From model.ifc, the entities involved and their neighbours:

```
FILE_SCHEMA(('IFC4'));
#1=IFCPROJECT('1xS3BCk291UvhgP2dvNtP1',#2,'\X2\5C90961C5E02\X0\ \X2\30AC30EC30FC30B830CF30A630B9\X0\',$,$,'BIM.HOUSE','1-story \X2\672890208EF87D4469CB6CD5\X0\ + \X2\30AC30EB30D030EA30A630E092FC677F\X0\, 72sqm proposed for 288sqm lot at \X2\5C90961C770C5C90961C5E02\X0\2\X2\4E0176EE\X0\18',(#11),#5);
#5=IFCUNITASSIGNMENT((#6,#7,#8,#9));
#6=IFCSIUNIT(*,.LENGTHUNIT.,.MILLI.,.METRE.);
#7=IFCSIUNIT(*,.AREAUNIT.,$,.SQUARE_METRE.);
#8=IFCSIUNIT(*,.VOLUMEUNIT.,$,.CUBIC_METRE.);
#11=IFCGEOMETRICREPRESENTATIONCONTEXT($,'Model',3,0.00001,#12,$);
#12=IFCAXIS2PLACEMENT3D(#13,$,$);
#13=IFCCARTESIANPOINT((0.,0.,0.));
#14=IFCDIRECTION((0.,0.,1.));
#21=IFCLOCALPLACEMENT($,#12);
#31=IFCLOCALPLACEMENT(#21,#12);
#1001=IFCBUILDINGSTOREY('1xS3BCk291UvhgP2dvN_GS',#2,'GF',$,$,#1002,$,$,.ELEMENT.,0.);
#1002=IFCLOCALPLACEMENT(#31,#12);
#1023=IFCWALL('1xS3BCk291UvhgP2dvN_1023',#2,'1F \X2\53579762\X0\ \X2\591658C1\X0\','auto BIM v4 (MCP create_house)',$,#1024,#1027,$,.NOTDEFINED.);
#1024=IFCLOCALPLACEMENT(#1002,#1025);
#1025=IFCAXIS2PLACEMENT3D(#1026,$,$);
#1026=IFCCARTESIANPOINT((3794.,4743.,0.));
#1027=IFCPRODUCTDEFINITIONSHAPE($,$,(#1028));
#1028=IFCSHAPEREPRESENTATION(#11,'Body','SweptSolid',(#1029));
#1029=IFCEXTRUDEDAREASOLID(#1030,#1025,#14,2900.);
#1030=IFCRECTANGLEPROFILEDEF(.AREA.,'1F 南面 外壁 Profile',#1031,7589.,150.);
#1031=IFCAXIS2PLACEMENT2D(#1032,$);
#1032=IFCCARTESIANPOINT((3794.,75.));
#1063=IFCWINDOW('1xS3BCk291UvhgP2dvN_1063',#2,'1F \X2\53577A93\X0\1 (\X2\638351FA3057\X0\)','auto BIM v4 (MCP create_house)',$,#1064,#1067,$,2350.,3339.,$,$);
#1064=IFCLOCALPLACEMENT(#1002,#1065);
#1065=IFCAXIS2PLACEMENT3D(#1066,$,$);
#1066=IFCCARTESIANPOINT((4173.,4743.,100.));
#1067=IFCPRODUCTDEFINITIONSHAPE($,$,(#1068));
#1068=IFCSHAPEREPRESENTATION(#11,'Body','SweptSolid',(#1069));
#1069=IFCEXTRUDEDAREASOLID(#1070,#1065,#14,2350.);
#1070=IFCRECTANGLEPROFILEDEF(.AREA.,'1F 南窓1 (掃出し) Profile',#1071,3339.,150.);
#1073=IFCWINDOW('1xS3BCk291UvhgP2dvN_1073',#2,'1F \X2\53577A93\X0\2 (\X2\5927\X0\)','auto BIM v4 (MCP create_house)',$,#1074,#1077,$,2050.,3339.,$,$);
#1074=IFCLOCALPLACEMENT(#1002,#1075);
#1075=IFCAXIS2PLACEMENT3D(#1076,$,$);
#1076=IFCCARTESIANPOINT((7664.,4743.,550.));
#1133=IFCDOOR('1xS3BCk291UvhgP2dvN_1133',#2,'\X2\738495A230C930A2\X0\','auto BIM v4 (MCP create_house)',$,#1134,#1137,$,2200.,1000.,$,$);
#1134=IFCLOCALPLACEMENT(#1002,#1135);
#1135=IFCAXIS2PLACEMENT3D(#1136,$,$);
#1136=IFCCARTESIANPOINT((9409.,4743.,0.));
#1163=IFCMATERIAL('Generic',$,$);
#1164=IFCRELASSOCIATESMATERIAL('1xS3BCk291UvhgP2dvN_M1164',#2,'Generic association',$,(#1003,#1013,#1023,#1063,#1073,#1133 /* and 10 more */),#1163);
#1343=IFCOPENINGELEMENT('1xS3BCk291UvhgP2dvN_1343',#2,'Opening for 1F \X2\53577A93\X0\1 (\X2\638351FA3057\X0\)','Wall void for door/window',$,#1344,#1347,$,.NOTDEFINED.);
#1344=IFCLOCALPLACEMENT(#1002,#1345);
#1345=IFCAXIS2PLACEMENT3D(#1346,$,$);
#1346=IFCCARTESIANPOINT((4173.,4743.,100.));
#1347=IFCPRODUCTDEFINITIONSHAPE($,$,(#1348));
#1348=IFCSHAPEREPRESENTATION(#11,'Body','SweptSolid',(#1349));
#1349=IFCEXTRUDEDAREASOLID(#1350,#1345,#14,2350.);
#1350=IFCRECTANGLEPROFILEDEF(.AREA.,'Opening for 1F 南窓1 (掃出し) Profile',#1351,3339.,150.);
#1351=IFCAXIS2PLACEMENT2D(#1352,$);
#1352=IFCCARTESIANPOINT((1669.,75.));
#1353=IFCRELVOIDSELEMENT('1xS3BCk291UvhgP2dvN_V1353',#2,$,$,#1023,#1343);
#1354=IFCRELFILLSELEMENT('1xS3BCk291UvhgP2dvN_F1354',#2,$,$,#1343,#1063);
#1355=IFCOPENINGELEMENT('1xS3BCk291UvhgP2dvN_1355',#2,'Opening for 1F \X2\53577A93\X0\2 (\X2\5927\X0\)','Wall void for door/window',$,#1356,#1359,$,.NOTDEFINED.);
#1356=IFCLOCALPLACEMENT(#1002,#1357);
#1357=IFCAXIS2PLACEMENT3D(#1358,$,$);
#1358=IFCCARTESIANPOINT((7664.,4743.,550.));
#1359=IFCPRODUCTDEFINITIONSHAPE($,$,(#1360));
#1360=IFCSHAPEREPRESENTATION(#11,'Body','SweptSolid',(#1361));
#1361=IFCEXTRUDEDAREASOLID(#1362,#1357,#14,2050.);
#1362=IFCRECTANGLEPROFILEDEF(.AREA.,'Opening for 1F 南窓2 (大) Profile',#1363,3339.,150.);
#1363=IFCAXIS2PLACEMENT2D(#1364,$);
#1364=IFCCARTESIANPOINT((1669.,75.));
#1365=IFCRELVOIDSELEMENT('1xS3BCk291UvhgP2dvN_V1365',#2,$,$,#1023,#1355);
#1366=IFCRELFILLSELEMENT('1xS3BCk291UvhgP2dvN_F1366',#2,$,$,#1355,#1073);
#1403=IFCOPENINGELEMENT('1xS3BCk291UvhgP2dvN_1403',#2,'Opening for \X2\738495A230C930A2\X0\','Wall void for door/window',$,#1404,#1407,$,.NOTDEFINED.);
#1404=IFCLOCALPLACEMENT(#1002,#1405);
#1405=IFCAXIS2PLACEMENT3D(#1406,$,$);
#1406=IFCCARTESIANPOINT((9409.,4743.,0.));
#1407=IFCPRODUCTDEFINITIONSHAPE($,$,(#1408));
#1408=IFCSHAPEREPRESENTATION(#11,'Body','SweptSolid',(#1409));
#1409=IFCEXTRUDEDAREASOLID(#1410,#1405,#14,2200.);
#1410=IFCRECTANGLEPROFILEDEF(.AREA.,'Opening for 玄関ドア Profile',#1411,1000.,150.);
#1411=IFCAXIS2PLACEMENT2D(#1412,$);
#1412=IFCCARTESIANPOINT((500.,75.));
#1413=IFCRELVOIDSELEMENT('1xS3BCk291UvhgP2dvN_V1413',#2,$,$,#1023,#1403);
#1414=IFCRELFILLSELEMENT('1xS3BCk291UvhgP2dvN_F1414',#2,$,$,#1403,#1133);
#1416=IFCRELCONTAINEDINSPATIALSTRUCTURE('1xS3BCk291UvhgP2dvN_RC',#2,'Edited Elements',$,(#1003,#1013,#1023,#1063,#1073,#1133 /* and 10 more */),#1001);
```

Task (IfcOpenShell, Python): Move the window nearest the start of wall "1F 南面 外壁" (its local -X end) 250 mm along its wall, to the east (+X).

```python
import ifcopenshell
import ifcopenshell.api.geometry
import ifcopenshell.util.placement
import ifcopenshell.util.unit

model = ifcopenshell.open("model.ifc")
unit_scale = ifcopenshell.util.unit.calculate_unit_scale(model)

window = model.by_guid("1xS3BCk291UvhgP2dvN_1063")
opening = window.FillsVoids[0].RelatingOpeningElement
wall = opening.VoidsElements[0].RelatingBuildingElement

wall_matrix = ifcopenshell.util.placement.get_local_placement(wall.ObjectPlacement)
shift = wall_matrix[:3, 0] * 0.25 / unit_scale
before = ifcopenshell.util.placement.get_local_placement(window.ObjectPlacement)[:3, 3].copy()

# The window is not placed relative to its opening, so move both.
for product in (opening, window):
    matrix = ifcopenshell.util.placement.get_local_placement(product.ObjectPlacement)
    matrix[:3, 3] += shift
    ifcopenshell.api.geometry.edit_object_placement(model, product=product, matrix=matrix, is_si=False)

after = ifcopenshell.util.placement.get_local_placement(window.ObjectPlacement)[:3, 3]
print("window moved by", (after - before).round(3) + 0.0)

model.write("model_updated.ifc")
```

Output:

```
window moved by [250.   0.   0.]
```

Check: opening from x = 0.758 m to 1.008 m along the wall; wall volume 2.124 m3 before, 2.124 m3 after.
